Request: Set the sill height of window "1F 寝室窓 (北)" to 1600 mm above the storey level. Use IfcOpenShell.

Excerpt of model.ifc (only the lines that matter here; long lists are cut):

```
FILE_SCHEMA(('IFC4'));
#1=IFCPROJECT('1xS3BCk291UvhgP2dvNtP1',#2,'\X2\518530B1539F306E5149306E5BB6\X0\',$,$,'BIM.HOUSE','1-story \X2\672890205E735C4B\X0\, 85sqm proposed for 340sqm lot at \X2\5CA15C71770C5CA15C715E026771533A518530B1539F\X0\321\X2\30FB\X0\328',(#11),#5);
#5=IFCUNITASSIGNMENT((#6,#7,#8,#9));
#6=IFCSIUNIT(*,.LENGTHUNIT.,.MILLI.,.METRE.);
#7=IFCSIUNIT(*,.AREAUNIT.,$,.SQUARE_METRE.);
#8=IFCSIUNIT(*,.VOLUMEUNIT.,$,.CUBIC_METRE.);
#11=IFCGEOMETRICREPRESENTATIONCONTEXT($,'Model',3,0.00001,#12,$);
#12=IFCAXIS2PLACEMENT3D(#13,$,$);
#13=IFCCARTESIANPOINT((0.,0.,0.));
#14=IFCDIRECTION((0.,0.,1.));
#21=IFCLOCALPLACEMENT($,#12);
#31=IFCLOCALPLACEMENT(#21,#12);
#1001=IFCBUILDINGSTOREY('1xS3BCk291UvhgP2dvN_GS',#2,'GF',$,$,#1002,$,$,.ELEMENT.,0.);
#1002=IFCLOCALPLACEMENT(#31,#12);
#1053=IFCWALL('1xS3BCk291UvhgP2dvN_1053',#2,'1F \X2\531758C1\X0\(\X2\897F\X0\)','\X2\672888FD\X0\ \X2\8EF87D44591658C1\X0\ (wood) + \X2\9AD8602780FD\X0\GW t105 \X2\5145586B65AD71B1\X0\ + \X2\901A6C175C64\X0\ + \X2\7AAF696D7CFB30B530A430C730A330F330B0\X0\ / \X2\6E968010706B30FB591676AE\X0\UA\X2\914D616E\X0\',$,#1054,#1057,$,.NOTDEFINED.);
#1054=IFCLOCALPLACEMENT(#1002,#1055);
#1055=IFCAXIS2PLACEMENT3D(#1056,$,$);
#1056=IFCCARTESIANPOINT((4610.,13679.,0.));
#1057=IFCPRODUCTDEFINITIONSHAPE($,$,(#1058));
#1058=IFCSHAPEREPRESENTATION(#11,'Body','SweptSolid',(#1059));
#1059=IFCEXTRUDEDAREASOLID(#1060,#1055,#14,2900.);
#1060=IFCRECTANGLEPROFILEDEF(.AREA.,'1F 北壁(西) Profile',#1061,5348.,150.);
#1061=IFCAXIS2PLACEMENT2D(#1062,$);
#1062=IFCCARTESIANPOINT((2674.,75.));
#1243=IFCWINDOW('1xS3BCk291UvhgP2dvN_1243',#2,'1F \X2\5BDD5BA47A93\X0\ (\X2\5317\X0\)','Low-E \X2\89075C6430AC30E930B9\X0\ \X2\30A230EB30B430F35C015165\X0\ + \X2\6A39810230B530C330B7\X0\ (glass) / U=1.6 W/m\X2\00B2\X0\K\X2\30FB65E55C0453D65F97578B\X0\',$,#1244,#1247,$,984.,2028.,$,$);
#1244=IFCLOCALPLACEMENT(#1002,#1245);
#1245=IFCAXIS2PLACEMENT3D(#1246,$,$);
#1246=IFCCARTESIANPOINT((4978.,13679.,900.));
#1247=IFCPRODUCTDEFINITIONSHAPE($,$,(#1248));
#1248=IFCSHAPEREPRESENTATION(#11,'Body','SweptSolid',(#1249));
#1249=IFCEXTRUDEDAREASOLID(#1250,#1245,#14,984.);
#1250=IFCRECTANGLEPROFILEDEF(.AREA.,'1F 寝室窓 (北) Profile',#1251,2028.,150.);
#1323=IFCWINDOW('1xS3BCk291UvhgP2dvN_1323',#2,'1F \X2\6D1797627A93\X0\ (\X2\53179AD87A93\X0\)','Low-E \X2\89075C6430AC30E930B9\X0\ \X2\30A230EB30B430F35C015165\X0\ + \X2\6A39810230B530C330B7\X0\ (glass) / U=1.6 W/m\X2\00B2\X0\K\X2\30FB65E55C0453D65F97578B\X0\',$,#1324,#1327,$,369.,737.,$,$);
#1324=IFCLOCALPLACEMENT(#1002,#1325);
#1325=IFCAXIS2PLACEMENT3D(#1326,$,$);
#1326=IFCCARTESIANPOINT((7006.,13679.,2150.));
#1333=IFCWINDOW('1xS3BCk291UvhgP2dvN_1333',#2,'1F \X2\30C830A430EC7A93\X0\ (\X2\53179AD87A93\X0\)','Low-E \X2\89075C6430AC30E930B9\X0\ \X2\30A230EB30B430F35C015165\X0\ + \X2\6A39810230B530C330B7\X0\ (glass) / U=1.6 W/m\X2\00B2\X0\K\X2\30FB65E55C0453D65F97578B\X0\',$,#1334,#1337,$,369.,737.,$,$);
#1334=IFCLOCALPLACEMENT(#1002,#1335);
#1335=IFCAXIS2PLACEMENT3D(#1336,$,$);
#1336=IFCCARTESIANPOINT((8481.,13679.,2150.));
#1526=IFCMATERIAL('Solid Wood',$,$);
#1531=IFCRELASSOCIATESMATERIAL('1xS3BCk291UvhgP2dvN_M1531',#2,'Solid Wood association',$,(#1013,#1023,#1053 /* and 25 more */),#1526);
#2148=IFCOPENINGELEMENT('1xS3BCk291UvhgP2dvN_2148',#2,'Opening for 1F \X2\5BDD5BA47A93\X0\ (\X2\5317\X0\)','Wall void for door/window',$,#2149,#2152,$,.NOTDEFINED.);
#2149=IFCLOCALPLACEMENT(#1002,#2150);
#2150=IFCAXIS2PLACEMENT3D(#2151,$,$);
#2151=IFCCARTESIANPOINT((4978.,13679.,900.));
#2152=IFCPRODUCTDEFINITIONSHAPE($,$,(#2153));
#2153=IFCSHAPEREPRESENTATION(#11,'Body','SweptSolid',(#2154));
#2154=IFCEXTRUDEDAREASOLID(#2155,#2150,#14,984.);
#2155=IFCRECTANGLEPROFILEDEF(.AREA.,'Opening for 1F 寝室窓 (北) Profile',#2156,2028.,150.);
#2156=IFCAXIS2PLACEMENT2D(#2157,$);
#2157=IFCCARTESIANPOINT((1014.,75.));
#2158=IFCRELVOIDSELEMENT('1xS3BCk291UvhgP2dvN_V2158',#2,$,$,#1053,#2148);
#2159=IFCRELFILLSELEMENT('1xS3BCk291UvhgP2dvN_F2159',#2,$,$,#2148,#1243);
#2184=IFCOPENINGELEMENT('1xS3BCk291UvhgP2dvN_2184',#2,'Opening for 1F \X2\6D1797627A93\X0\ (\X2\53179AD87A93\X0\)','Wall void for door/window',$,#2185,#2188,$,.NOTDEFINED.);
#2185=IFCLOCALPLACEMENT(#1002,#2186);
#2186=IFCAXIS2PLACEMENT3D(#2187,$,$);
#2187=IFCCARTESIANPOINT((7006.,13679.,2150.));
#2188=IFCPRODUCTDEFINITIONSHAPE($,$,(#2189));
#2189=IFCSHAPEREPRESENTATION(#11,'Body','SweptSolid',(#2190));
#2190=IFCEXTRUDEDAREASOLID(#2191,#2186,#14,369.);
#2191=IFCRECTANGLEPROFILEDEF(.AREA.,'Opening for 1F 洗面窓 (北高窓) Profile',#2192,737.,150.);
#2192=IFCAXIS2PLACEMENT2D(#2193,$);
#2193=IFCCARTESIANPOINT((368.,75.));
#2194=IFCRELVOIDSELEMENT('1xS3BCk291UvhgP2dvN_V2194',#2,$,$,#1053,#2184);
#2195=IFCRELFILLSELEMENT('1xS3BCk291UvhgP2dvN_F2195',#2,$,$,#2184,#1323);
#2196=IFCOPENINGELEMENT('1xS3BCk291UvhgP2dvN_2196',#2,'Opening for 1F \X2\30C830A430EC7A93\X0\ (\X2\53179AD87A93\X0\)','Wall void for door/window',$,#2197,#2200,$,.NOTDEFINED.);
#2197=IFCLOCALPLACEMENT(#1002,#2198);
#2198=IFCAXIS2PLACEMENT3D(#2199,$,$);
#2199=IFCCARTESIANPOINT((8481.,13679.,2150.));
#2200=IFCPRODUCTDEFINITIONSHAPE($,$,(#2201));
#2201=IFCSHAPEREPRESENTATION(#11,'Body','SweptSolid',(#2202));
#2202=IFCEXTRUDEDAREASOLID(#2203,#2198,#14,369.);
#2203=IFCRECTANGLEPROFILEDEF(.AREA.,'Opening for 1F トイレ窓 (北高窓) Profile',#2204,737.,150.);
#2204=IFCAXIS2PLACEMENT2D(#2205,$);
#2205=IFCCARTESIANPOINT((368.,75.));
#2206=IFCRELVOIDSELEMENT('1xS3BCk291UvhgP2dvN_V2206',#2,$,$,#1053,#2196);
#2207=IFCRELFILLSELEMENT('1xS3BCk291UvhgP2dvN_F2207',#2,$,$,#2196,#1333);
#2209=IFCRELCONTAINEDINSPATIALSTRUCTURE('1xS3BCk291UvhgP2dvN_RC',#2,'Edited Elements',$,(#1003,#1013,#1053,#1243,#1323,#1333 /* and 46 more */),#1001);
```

```python
import numpy as np
import ifcopenshell
import ifcopenshell.api.geometry
import ifcopenshell.geom
import ifcopenshell.util.element
import ifcopenshell.util.placement
import ifcopenshell.util.shape
import ifcopenshell.util.unit

model = ifcopenshell.open("model.ifc")
unit_scale = ifcopenshell.util.unit.calculate_unit_scale(model)

window = model.by_id(1243)
opening = window.FillsVoids[0].RelatingOpeningElement
storey = ifcopenshell.util.element.get_container(window, ifc_class="IfcBuildingStorey")
level = ifcopenshell.util.placement.get_local_placement(storey.ObjectPlacement)[2, 3]

# The opening's origin need not be at the sill, so measure its lowest point.
shape = ifcopenshell.geom.create_shape(ifcopenshell.geom.settings(), opening)
bottom = ifcopenshell.util.shape.get_shape_bottom_elevation(shape, shape.geometry) / unit_scale
dz = level + 1.6 / unit_scale - bottom

shift = np.array([0.0, 0.0, dz])
# The window is not placed relative to its opening, so move both.
for product in (opening, window):
    matrix = ifcopenshell.util.placement.get_local_placement(product.ObjectPlacement)
    matrix[:3, 3] += shift
    ifcopenshell.api.geometry.edit_object_placement(model, product=product, matrix=matrix, is_si=False)

print(f"moved by {dz * unit_scale:+.3f} m")

model.write("model_edited.ifc")
```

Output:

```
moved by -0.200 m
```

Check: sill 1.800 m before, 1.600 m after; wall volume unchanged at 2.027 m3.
